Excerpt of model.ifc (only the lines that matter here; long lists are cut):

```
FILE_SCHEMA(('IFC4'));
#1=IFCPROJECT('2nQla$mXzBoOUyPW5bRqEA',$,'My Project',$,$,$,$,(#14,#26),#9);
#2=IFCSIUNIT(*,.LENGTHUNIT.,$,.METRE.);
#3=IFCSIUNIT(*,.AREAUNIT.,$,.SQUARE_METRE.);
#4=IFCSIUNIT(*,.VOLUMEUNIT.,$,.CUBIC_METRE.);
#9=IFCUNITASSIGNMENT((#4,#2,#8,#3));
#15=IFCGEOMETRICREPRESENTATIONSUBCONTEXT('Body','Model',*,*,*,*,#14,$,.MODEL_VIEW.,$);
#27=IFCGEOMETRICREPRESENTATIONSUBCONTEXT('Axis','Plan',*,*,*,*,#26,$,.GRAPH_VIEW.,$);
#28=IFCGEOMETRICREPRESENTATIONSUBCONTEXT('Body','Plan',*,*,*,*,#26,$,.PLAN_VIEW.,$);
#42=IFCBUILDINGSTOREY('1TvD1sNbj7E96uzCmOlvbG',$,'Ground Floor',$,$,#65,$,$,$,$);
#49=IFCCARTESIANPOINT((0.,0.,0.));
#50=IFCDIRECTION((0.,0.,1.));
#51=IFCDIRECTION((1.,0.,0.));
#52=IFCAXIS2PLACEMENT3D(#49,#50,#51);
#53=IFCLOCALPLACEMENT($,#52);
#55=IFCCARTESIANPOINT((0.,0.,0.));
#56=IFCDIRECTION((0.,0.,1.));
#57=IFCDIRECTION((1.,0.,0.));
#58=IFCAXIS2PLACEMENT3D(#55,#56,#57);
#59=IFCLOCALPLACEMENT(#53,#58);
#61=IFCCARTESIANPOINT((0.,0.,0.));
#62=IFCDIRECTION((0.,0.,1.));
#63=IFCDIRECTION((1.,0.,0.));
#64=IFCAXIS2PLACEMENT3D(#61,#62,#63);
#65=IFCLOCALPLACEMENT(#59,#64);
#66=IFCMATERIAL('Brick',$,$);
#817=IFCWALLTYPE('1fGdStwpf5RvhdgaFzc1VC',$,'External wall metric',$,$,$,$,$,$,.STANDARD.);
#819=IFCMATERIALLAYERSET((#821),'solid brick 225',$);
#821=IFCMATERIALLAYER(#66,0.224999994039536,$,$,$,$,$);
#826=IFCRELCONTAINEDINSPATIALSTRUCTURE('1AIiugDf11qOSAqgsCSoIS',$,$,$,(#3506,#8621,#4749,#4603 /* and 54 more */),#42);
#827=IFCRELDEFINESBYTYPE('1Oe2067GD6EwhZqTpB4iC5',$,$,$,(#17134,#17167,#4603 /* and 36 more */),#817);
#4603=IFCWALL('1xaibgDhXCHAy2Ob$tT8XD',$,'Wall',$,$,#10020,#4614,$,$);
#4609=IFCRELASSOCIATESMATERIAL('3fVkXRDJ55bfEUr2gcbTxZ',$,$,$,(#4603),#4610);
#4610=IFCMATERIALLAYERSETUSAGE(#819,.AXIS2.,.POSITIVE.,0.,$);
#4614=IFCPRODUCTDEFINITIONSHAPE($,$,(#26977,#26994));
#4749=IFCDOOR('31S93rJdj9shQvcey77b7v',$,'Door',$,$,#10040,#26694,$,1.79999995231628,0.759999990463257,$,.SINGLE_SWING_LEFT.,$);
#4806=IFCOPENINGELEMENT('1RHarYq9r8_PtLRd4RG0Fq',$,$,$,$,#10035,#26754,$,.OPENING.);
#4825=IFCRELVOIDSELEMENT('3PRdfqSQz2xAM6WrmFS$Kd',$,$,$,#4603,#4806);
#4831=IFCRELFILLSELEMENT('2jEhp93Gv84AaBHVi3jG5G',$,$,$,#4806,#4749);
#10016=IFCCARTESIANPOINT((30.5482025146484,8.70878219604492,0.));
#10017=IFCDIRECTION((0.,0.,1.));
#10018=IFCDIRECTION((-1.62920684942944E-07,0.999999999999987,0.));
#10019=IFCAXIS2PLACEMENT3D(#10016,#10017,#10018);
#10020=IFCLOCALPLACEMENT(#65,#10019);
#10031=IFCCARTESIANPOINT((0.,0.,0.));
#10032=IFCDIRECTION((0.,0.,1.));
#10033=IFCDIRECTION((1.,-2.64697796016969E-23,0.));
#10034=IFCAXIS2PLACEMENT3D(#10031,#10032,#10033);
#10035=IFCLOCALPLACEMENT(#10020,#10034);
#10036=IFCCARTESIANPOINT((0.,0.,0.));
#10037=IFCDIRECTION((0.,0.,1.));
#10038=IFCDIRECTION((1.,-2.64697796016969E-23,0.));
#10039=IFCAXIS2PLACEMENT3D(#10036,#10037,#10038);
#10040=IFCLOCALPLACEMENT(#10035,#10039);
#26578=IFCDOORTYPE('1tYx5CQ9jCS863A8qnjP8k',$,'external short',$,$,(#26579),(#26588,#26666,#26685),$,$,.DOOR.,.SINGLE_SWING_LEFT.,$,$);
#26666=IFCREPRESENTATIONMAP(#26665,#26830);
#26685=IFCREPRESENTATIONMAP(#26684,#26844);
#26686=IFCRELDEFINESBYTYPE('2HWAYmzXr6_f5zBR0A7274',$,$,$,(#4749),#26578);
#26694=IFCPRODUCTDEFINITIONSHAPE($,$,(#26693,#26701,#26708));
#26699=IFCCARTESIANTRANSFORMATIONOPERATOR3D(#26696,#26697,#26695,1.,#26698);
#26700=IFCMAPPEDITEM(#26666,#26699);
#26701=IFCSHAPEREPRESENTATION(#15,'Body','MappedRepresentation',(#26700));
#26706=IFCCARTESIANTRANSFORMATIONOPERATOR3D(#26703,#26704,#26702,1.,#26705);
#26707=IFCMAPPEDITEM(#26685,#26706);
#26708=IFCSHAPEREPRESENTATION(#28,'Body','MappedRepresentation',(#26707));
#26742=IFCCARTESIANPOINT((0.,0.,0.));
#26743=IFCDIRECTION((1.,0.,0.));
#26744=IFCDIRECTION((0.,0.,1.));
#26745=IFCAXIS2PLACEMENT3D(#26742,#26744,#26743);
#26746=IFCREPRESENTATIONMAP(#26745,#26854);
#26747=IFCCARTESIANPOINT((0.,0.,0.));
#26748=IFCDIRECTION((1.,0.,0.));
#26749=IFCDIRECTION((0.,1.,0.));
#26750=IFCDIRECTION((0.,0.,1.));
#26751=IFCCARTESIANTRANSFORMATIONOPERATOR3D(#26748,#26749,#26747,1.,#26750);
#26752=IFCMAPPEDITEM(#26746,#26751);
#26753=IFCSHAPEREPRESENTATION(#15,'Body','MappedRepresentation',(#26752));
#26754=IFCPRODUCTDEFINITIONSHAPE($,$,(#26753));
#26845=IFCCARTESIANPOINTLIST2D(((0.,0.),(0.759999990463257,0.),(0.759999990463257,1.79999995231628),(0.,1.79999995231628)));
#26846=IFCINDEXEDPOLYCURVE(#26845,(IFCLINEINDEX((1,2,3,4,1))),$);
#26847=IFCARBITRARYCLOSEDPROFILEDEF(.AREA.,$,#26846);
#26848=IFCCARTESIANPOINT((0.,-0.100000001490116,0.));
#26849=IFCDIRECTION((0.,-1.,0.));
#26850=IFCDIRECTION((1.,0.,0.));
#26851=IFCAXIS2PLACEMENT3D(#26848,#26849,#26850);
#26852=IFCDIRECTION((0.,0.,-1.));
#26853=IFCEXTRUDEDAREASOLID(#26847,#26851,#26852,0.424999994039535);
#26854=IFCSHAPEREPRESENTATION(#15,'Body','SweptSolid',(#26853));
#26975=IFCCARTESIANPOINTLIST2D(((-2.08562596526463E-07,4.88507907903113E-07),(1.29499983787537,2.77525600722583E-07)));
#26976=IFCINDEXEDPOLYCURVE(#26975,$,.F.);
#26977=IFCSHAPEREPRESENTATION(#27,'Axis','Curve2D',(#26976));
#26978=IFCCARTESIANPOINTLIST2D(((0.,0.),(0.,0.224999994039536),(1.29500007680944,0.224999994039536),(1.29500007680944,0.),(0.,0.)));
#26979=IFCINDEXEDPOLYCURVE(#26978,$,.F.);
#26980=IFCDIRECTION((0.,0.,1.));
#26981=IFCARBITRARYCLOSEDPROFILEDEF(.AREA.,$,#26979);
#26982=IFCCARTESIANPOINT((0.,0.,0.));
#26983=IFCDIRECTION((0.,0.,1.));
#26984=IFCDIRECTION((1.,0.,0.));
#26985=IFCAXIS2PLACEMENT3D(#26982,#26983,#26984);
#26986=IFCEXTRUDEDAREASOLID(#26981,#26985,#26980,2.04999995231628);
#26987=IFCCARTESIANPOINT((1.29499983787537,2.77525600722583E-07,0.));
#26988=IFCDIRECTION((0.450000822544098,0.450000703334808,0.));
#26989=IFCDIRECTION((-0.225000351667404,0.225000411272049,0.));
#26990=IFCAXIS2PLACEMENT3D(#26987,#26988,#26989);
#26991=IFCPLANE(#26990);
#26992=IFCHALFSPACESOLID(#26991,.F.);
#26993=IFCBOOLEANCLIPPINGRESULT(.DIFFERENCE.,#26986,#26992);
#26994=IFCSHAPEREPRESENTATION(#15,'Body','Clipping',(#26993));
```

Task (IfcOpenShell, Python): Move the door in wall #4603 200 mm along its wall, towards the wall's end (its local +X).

```python
import ifcopenshell
import ifcopenshell.api.geometry
import ifcopenshell.util.placement
import ifcopenshell.util.unit

model = ifcopenshell.open("model.ifc")
unit_scale = ifcopenshell.util.unit.calculate_unit_scale(model)

door = model.by_id(4749)
opening = door.FillsVoids[0].RelatingOpeningElement
wall = opening.VoidsElements[0].RelatingBuildingElement

wall_matrix = ifcopenshell.util.placement.get_local_placement(wall.ObjectPlacement)
shift = wall_matrix[:3, 0] * 0.2 / unit_scale
before = ifcopenshell.util.placement.get_local_placement(door.ObjectPlacement)[:3, 3].copy()

# The door is placed relative to its opening, so it follows when the opening moves.
matrix = ifcopenshell.util.placement.get_local_placement(opening.ObjectPlacement)
matrix[:3, 3] += shift
ifcopenshell.api.geometry.edit_object_placement(
    model, product=opening, matrix=matrix, is_si=False, should_transform_children=True
)

after = ifcopenshell.util.placement.get_local_placement(door.ObjectPlacement)[:3, 3]
print("door moved by", (after - before).round(3) + 0.0)

model.write("model_v2.ifc")
```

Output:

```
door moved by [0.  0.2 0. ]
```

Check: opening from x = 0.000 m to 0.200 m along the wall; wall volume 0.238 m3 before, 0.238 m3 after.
